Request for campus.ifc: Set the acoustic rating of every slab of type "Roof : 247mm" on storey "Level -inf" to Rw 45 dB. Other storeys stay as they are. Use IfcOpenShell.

First a look at what the model holds.

```python
import ifcopenshell
import ifcopenshell.util.element

model = ifcopenshell.open("campus.ifc")
print(model.schema)
storey = next(s for s in model.by_type("IfcBuildingStorey") if s.Name == "Level -inf")
slabs = [e for e in ifcopenshell.util.element.get_decomposition(storey) if e.is_a("IfcSlab")]
seen = {}
for e in slabs:
    element_type = ifcopenshell.util.element.get_type(e)
    key = (element_type.Name if element_type != e and element_type else None, ifcopenshell.util.element.get_pset(e, "Pset_SlabCommon", "AcousticRating"))
    seen[key] = seen.get(key, 0) + 1
for (name, value), count in sorted(seen.items(), key=str):
    print(count, "x", name, "|", value)
```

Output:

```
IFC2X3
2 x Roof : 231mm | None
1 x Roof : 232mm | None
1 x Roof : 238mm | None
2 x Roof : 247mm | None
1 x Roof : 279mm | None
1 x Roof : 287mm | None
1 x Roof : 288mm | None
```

```python
import ifcopenshell
import ifcopenshell.api.pset
import ifcopenshell.util.element

model = ifcopenshell.open("campus.ifc")

storey = next(s for s in model.by_type("IfcBuildingStorey") if s.Name == "Level -inf")
slabs = [e for e in ifcopenshell.util.element.get_decomposition(storey) if e.is_a("IfcSlab")]

count = 0
for e in slabs:
    element_type = ifcopenshell.util.element.get_type(e)
    if element_type in (None, e) or element_type.Name != "Roof : 247mm":
        continue
    # add_pset returns the element's existing set when there is one.
    pset = ifcopenshell.api.pset.add_pset(model, product=e, name="Pset_SlabCommon")
    ifcopenshell.api.pset.edit_pset(model, pset=pset, properties={"AcousticRating": "Rw 45 dB"})
    count += 1

print(count, "slabs updated")

model.write("campus-out.ifc")
```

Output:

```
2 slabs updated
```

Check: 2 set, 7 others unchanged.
